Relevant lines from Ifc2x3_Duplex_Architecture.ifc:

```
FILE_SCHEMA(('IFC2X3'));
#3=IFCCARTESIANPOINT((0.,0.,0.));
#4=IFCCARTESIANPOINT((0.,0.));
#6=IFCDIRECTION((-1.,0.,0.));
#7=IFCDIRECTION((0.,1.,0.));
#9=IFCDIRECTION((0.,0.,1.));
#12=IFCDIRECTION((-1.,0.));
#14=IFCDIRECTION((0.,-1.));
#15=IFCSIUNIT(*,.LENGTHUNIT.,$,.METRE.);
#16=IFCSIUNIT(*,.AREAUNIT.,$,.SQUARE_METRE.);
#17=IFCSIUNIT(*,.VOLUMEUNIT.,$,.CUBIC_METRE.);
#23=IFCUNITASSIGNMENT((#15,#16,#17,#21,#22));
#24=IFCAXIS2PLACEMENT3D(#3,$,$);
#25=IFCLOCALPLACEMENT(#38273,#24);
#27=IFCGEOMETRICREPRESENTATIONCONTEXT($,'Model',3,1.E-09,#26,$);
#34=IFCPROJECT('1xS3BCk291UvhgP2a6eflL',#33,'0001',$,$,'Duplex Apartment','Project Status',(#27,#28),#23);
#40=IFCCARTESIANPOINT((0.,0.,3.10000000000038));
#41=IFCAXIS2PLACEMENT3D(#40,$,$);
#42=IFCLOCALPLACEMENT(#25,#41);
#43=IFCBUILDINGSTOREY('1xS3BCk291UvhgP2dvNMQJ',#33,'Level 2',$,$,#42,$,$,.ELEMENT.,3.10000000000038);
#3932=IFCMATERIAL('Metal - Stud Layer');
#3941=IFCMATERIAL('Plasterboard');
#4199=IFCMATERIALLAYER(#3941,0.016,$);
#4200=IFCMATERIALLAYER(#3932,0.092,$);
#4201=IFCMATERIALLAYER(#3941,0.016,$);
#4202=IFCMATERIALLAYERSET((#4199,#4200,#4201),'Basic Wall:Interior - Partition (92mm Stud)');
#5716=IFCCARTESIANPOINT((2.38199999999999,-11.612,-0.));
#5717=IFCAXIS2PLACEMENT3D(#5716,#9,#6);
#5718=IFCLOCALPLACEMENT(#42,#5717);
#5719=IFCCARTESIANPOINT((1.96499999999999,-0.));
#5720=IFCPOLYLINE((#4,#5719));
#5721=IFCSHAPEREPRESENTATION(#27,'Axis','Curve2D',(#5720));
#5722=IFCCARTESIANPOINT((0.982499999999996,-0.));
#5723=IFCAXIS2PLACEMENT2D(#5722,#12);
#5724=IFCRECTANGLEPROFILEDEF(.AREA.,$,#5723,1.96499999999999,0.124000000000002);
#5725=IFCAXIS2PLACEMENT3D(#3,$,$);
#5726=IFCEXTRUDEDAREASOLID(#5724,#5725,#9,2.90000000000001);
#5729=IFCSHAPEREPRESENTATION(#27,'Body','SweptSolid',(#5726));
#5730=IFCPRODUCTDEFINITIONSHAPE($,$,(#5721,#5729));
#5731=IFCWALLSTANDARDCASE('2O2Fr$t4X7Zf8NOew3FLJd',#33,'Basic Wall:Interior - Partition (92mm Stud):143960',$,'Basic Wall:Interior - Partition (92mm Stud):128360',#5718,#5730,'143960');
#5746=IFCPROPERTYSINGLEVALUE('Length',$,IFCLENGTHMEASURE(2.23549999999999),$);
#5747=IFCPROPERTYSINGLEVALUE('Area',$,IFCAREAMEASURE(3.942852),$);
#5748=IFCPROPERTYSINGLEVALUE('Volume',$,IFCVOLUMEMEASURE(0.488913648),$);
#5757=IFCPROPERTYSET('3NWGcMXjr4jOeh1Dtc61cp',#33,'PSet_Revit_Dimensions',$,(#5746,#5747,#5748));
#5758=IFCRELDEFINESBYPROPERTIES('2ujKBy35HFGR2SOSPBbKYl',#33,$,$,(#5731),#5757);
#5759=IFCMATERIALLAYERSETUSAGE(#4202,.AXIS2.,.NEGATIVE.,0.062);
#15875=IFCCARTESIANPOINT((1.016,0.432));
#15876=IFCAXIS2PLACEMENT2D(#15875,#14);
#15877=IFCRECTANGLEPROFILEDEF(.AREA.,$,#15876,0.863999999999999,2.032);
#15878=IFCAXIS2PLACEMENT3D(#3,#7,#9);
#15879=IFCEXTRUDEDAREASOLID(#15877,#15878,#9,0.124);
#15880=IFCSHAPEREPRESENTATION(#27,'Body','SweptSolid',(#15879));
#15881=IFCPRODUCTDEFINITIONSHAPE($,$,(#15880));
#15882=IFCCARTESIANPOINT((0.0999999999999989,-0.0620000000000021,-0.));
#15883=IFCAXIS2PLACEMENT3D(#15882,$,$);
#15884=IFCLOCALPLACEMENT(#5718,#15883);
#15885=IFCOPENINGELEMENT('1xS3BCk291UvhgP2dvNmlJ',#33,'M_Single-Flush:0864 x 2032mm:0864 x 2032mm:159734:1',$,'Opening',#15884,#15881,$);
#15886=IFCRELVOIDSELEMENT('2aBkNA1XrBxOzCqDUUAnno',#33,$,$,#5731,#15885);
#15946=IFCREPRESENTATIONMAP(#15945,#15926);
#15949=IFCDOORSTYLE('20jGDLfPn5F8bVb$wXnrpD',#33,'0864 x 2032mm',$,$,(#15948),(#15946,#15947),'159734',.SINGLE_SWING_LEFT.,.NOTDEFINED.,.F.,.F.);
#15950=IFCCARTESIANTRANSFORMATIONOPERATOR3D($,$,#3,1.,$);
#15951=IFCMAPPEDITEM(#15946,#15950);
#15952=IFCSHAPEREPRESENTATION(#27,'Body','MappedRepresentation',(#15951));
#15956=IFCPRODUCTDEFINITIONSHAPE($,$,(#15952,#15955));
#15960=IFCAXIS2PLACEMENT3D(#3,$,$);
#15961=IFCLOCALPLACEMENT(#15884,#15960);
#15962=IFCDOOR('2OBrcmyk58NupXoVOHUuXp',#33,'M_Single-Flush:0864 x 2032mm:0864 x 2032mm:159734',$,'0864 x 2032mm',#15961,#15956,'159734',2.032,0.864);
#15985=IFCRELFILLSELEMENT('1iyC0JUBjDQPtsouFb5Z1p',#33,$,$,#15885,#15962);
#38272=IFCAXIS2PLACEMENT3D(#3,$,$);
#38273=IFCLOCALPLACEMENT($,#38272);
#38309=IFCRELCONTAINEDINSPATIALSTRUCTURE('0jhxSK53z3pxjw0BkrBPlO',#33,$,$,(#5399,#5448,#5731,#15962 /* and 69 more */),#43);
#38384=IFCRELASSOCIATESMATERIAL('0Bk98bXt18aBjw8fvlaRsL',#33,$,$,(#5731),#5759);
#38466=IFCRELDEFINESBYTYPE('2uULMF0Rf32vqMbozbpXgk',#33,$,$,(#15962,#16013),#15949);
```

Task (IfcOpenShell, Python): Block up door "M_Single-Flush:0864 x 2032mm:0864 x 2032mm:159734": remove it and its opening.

```python
import ifcopenshell
import ifcopenshell.api.feature
import ifcopenshell.api.pset
import ifcopenshell.api.root
import ifcopenshell.geom
import ifcopenshell.util.element
import ifcopenshell.util.shape
import ifcopenshell.util.unit

model = ifcopenshell.open("Ifc2x3_Duplex_Architecture.ifc")
area_scale = ifcopenshell.util.unit.calculate_unit_scale(model, "AREAUNIT")
volume_scale = ifcopenshell.util.unit.calculate_unit_scale(model, "VOLUMEUNIT")
settings = ifcopenshell.geom.settings()


def volume(element):
    """Net volume in cubic metres, openings subtracted."""
    shape = ifcopenshell.geom.create_shape(settings, element)
    return ifcopenshell.util.shape.get_volume(shape.geometry)


door = model.by_id(15962)
opening = door.FillsVoids[0].RelatingOpeningElement
wall = opening.VoidsElements[0].RelatingBuildingElement
before = volume(wall)

ifcopenshell.api.root.remove_product(model, product=door)
ifcopenshell.api.feature.remove_feature(model, feature=opening)

after = volume(wall)
thickness = 0.124  # wall thickness in metres

# Update the wall's stored quantities.
pset = model.by_id(ifcopenshell.util.element.get_pset(wall, "PSet_Revit_Dimensions", should_inherit=False)["id"])
ifcopenshell.api.pset.edit_pset(model, pset=pset, properties={
    "Area": model.create_entity("IfcAreaMeasure", after / thickness / area_scale),
    "Volume": model.create_entity("IfcVolumeMeasure", after / volume_scale),
})

print(f"wall volume {before:.3f} -> {after:.3f} m3")

model.write("Ifc2x3_Duplex_Architecture_v2.ifc")
```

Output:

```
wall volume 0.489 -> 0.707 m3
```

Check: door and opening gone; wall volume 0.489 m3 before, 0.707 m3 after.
